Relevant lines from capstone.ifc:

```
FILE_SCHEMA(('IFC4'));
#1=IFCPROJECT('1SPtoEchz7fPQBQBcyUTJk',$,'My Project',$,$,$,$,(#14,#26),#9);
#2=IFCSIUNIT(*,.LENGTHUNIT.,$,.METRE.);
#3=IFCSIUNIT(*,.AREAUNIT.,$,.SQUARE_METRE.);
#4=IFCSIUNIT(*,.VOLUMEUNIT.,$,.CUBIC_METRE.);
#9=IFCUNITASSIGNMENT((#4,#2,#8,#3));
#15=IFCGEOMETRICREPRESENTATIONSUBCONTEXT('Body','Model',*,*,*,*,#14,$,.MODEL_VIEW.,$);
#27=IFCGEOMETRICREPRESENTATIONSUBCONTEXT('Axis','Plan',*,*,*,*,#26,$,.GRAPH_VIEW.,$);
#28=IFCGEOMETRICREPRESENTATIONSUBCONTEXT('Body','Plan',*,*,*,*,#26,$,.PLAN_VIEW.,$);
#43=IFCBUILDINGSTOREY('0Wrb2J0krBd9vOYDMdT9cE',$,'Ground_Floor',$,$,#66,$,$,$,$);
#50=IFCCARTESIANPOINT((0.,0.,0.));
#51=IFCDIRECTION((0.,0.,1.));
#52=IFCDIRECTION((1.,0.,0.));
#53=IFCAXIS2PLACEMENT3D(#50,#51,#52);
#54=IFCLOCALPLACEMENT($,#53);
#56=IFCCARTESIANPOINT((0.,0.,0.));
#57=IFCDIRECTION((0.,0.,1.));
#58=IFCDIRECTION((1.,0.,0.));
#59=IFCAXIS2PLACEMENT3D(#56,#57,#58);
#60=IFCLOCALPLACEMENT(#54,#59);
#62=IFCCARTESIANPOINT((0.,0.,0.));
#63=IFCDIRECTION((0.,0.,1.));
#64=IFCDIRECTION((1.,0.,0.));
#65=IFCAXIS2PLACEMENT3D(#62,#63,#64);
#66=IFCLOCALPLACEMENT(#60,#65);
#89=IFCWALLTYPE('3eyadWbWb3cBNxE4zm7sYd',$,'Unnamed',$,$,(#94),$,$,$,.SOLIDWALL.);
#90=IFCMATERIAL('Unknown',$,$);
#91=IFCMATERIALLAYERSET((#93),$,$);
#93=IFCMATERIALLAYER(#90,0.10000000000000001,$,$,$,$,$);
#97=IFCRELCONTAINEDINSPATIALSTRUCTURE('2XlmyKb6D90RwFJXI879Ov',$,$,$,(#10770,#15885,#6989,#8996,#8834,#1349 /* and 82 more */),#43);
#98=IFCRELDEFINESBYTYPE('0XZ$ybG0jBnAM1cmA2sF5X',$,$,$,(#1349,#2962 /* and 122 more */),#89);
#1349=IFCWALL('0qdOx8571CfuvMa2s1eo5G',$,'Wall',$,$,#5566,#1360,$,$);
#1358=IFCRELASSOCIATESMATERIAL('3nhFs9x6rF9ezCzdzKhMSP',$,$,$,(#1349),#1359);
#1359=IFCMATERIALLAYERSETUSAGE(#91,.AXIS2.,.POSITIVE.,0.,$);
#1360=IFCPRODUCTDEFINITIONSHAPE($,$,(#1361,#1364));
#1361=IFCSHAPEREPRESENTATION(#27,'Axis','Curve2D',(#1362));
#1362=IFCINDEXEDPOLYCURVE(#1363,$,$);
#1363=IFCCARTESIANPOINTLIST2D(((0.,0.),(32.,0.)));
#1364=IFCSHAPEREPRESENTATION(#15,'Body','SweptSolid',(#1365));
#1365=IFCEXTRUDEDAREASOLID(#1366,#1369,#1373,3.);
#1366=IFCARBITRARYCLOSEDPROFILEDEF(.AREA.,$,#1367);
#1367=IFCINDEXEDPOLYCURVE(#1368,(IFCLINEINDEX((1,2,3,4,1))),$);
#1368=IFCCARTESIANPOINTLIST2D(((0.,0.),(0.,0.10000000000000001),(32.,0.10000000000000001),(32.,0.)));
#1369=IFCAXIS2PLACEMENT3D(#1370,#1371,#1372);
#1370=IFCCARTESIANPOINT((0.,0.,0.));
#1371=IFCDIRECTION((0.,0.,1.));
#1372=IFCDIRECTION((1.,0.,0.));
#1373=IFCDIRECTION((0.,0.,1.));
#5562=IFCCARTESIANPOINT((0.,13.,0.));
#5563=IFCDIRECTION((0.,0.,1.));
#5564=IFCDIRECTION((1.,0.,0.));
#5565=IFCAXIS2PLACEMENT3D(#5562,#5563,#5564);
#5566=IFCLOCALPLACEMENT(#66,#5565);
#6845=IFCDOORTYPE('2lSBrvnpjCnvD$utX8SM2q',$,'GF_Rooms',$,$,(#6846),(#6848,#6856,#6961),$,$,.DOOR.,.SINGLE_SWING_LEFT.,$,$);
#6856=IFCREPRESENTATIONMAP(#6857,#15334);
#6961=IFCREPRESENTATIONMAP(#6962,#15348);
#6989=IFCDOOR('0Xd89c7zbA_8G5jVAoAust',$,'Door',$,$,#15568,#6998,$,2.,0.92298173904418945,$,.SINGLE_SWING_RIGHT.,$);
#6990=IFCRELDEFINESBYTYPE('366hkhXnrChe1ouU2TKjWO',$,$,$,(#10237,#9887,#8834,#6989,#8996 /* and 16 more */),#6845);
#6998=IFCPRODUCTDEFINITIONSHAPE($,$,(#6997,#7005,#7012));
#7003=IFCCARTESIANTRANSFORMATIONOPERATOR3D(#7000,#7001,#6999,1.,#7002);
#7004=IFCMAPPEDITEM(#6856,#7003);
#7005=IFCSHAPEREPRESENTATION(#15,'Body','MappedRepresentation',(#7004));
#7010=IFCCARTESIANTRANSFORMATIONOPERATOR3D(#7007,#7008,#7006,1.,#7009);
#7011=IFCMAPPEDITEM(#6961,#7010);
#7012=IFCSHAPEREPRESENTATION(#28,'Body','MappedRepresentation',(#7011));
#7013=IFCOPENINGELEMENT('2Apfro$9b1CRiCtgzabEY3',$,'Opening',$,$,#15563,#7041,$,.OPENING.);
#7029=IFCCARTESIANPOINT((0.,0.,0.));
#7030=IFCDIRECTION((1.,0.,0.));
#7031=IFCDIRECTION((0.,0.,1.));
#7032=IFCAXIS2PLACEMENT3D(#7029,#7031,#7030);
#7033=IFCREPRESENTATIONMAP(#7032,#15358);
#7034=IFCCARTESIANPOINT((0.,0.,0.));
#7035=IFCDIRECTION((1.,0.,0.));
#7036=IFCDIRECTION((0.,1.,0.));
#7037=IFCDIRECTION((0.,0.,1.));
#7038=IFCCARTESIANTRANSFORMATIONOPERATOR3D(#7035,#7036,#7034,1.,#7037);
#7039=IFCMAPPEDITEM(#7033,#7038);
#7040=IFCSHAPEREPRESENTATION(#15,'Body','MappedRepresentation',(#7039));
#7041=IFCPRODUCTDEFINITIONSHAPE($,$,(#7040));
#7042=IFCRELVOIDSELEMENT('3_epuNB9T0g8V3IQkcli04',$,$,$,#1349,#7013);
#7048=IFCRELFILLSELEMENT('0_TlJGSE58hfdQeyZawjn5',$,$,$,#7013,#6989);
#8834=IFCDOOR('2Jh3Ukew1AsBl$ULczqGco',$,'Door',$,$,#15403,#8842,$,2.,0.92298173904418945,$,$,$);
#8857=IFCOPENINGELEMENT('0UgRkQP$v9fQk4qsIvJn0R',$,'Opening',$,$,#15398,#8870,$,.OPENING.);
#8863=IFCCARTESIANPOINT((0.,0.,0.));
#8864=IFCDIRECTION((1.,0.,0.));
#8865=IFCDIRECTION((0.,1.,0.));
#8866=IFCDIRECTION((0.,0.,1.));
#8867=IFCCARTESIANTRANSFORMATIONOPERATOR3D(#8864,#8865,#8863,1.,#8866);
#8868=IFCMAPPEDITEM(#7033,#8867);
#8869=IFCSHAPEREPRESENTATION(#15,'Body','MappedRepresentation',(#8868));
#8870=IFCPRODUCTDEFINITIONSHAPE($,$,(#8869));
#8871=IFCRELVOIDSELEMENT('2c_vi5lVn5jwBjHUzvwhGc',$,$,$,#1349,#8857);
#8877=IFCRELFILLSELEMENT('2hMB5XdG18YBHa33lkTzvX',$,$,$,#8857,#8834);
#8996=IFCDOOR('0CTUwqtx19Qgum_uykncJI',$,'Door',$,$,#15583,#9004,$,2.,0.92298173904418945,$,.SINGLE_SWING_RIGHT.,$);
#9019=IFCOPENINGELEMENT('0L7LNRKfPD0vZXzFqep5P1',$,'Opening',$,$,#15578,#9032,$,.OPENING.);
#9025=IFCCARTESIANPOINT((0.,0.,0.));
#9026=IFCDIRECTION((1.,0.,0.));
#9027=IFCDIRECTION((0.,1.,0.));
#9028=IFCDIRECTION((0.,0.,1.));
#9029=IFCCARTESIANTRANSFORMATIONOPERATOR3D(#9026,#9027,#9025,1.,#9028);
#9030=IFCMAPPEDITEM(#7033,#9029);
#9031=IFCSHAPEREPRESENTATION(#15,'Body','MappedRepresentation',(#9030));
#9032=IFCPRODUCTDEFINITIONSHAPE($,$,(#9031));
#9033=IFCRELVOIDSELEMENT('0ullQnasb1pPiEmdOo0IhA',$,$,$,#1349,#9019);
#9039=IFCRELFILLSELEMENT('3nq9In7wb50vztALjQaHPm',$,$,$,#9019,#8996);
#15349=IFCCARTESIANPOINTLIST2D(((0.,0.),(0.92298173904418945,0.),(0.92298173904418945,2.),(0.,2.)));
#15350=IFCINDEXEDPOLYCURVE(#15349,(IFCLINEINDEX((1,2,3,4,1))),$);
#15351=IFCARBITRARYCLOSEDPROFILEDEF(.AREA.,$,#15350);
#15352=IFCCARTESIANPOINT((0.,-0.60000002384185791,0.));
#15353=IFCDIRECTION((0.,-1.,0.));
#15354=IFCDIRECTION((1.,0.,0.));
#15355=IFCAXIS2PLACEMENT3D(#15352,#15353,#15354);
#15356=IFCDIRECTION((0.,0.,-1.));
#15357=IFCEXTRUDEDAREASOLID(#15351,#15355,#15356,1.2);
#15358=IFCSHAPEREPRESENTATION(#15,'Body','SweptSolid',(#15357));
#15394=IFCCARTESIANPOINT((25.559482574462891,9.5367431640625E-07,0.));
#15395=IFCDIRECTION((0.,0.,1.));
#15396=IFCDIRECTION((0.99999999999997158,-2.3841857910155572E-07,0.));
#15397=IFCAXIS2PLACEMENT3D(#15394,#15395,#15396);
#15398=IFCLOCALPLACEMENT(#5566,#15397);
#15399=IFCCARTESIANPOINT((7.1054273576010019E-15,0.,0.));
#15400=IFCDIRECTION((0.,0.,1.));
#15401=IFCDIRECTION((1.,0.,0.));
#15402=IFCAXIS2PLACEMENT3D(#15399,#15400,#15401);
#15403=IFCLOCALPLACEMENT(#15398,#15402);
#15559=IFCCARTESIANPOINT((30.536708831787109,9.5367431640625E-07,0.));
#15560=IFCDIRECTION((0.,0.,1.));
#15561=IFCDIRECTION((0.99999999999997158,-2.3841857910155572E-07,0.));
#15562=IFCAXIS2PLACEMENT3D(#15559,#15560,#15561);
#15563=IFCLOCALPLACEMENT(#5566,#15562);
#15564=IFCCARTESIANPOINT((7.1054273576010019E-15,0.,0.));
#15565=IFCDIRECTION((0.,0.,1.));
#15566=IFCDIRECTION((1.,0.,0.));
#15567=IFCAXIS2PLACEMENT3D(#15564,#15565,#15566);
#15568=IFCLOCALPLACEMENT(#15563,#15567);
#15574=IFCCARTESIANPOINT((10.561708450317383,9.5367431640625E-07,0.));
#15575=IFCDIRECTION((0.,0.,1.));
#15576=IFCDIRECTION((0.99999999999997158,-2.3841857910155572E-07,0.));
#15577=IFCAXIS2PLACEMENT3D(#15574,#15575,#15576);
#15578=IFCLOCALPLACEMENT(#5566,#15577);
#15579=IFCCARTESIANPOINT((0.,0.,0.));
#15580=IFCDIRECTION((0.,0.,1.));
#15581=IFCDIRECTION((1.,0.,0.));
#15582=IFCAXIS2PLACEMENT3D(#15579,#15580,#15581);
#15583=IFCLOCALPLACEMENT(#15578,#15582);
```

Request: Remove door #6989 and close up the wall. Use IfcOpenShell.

```python
import ifcopenshell
import ifcopenshell.api.feature
import ifcopenshell.api.root
import ifcopenshell.geom
import ifcopenshell.util.shape

model = ifcopenshell.open("capstone.ifc")
settings = ifcopenshell.geom.settings()


def volume(element):
    """Net volume in cubic metres, openings subtracted."""
    shape = ifcopenshell.geom.create_shape(settings, element)
    return ifcopenshell.util.shape.get_volume(shape.geometry)


door = model.by_guid("0Xd89c7zbA_8G5jVAoAust")
opening = door.FillsVoids[0].RelatingOpeningElement
wall = opening.VoidsElements[0].RelatingBuildingElement
before = volume(wall)

ifcopenshell.api.root.remove_product(model, product=door)
ifcopenshell.api.feature.remove_feature(model, feature=opening)

after = volume(wall)

print(f"wall volume {before:.3f} -> {after:.3f} m3")

model.write("capstone_v2.ifc")
```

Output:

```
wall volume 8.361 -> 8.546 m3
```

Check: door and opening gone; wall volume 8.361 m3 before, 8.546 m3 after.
